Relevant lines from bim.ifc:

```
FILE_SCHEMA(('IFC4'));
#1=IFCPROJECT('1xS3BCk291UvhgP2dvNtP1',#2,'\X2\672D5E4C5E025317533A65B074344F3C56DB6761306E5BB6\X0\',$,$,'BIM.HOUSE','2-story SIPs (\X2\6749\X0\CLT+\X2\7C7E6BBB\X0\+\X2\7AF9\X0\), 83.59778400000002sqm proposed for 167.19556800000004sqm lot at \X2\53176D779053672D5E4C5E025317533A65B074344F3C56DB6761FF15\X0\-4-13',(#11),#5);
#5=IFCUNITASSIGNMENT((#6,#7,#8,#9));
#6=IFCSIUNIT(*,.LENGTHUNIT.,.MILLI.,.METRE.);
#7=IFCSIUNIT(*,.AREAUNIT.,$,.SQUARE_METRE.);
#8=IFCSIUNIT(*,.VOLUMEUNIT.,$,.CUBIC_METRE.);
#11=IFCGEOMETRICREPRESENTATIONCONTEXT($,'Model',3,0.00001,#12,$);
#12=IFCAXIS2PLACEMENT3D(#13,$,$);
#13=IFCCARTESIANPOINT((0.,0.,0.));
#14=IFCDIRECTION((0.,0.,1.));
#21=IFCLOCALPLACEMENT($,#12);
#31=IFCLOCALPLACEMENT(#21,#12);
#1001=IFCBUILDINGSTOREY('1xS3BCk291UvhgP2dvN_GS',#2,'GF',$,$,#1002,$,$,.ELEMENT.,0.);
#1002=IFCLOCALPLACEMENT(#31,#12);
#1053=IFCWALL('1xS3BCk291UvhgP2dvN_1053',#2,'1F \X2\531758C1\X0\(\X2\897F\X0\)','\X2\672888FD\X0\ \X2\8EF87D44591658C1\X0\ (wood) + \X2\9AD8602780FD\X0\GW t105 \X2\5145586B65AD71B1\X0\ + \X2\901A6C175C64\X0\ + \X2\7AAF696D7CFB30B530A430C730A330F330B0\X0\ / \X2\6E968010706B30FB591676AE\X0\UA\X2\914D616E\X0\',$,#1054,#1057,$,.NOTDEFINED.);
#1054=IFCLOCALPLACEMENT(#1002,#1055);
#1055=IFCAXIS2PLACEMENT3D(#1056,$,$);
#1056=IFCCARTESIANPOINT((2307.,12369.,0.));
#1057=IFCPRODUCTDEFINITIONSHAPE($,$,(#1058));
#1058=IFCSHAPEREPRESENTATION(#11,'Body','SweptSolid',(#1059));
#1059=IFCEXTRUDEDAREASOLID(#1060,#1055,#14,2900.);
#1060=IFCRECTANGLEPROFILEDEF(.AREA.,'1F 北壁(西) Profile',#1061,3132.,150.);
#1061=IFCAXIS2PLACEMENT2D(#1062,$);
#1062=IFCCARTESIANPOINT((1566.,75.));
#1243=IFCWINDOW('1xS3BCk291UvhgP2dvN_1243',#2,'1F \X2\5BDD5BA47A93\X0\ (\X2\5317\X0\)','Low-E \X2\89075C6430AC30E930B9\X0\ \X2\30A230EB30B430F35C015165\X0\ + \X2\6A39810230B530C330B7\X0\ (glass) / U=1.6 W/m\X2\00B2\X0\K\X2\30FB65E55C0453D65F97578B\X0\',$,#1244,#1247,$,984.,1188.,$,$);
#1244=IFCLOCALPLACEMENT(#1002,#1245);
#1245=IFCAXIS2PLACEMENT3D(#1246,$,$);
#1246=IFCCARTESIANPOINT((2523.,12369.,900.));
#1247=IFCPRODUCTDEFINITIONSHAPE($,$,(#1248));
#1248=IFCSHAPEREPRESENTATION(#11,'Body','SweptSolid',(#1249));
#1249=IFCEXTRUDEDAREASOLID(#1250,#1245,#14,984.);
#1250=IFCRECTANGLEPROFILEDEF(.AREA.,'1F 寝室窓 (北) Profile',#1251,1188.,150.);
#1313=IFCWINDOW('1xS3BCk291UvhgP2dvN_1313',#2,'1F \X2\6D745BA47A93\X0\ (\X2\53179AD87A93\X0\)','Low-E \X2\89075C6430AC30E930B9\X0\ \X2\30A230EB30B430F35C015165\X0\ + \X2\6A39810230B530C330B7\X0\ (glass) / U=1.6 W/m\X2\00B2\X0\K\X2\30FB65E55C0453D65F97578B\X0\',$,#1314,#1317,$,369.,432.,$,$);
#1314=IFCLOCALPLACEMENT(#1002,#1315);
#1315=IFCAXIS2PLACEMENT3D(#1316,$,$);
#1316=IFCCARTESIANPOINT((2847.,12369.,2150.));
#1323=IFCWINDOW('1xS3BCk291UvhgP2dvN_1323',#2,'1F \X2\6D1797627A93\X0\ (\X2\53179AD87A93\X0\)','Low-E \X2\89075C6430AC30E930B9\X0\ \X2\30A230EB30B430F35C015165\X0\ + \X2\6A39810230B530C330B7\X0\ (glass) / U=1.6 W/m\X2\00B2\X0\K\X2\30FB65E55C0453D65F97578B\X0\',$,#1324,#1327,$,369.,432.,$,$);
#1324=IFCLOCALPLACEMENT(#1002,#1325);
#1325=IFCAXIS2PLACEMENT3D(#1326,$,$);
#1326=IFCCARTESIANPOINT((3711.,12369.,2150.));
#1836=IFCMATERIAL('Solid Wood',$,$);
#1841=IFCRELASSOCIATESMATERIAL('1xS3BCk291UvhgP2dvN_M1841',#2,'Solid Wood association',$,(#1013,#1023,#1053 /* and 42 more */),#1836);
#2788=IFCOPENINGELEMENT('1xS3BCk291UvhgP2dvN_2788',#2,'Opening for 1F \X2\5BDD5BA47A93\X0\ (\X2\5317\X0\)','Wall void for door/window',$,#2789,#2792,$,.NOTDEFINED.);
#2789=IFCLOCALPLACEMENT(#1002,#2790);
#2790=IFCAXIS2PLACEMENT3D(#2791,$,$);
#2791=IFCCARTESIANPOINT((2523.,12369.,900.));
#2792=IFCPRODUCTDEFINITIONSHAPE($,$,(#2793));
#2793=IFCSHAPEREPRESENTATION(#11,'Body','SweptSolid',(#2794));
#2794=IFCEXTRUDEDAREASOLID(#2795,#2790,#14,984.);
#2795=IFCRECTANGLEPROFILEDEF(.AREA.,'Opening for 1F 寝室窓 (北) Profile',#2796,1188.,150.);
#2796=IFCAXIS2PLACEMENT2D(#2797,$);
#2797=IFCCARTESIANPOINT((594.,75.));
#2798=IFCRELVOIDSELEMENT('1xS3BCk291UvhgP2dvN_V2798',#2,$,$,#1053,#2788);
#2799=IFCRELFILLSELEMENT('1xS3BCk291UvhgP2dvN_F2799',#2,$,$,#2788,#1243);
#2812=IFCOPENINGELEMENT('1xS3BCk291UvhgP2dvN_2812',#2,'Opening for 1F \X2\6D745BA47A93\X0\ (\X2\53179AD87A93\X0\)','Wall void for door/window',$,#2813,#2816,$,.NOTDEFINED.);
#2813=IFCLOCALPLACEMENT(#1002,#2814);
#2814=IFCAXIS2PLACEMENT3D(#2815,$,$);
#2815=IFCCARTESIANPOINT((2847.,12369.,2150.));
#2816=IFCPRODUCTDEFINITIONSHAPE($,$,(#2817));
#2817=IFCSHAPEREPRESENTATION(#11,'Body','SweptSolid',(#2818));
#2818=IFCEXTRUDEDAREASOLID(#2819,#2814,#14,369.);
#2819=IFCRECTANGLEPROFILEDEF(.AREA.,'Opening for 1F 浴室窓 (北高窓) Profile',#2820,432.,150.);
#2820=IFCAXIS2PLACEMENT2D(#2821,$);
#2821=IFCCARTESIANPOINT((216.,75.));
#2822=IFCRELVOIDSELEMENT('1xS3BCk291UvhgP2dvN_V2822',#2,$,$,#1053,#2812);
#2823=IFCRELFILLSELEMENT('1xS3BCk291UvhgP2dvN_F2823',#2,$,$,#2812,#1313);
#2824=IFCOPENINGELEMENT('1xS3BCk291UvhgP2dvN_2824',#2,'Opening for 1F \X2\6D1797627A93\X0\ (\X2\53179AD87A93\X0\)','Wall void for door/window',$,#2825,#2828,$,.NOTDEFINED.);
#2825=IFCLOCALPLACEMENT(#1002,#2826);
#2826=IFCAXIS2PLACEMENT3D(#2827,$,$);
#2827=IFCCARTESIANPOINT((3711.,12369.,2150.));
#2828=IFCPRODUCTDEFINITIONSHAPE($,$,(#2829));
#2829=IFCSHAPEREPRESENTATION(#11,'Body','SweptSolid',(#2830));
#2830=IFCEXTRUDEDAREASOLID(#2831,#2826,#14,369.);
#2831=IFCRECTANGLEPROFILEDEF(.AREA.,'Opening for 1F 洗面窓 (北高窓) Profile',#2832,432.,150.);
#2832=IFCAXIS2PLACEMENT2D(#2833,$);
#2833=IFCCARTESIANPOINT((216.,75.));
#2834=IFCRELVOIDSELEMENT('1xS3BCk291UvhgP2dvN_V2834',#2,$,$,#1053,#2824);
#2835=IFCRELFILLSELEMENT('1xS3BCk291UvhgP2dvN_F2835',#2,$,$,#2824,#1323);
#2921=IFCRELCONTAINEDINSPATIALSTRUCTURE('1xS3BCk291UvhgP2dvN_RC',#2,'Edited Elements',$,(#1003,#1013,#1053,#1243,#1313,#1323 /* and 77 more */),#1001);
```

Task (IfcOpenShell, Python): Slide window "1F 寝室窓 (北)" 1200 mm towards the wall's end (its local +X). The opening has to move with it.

```python
import ifcopenshell
import ifcopenshell.api.geometry
import ifcopenshell.util.placement
import ifcopenshell.util.unit

model = ifcopenshell.open("bim.ifc")
unit_scale = ifcopenshell.util.unit.calculate_unit_scale(model)

window = model.by_id(1243)
opening = window.FillsVoids[0].RelatingOpeningElement
wall = opening.VoidsElements[0].RelatingBuildingElement

wall_matrix = ifcopenshell.util.placement.get_local_placement(wall.ObjectPlacement)
shift = wall_matrix[:3, 0] * 1.2 / unit_scale
before = ifcopenshell.util.placement.get_local_placement(window.ObjectPlacement)[:3, 3].copy()

# The window is not placed relative to its opening, so move both.
for product in (opening, window):
    matrix = ifcopenshell.util.placement.get_local_placement(product.ObjectPlacement)
    matrix[:3, 3] += shift
    ifcopenshell.api.geometry.edit_object_placement(model, product=product, matrix=matrix, is_si=False)

after = ifcopenshell.util.placement.get_local_placement(window.ObjectPlacement)[:3, 3]
print("window moved by", (after - before).round(3) + 0.0)

model.write("bim_updated.ifc")
```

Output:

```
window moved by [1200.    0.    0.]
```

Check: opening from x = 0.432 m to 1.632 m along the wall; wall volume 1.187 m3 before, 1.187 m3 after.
